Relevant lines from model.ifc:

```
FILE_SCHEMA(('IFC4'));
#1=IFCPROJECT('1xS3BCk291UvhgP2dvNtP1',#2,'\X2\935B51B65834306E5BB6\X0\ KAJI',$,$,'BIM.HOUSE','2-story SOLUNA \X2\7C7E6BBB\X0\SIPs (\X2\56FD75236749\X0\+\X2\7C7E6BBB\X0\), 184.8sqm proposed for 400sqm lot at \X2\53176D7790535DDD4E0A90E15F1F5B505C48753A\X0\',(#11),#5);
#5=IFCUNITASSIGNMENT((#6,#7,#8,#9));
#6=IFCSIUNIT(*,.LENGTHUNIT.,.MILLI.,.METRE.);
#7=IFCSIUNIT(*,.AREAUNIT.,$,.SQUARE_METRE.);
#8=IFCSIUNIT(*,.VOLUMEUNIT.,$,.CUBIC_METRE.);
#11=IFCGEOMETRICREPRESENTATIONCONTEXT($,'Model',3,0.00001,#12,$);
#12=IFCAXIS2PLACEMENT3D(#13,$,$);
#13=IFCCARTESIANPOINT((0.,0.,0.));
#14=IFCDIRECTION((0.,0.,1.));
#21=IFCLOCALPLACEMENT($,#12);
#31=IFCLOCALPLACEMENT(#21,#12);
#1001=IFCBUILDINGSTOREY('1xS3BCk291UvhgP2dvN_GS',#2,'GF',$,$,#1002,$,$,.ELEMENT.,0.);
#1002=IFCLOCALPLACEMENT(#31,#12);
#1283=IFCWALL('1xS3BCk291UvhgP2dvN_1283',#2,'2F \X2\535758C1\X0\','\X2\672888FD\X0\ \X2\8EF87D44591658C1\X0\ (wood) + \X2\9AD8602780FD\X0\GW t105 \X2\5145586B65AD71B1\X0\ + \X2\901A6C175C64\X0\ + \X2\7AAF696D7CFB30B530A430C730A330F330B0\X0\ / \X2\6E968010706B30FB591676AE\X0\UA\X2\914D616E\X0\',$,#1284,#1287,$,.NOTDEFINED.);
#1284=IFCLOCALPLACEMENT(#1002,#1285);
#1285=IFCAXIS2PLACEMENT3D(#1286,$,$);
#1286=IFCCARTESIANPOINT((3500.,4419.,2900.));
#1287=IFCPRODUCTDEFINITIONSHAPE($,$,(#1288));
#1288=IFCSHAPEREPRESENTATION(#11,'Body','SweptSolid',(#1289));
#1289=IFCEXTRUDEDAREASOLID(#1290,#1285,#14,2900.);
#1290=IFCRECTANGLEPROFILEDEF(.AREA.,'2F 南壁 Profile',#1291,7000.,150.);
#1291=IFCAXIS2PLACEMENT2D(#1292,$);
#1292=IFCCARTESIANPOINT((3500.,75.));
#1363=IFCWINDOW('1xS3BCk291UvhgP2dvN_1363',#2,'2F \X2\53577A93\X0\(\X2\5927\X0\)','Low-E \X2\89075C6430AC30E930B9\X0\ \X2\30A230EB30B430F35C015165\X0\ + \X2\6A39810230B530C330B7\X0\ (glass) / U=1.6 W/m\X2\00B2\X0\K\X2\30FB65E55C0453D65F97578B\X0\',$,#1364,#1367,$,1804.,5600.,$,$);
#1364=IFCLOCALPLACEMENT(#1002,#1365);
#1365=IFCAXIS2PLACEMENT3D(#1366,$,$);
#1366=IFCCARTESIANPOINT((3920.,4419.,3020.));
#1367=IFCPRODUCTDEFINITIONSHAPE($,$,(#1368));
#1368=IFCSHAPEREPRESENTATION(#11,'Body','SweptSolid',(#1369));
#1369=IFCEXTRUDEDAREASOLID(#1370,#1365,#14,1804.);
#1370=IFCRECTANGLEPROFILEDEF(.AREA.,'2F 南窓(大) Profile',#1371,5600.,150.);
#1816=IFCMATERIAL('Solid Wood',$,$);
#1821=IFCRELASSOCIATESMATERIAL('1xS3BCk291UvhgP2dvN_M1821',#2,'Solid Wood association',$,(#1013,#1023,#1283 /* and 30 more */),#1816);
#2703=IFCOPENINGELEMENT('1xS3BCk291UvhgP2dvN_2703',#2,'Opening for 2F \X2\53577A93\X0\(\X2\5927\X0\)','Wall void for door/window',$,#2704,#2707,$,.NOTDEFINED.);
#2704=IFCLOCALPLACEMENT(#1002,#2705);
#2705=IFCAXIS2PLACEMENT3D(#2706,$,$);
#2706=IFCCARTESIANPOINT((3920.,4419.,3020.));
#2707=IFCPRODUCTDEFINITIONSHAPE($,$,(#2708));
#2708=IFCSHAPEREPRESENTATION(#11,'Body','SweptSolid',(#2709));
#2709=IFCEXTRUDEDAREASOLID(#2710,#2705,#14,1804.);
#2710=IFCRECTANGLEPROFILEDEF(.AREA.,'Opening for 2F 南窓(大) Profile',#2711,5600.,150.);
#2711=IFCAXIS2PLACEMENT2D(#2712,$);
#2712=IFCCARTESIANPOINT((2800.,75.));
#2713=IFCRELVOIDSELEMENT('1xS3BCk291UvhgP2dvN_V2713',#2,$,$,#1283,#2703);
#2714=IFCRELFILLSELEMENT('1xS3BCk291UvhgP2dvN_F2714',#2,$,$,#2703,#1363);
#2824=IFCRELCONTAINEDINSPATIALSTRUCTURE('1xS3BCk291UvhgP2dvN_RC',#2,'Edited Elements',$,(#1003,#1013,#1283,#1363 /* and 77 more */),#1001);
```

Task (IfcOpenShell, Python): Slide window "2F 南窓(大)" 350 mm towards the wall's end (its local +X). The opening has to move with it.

```python
import ifcopenshell
import ifcopenshell.api.geometry
import ifcopenshell.util.placement
import ifcopenshell.util.unit

model = ifcopenshell.open("model.ifc")
unit_scale = ifcopenshell.util.unit.calculate_unit_scale(model)

window = model.by_guid("1xS3BCk291UvhgP2dvN_1363")
opening = window.FillsVoids[0].RelatingOpeningElement
wall = opening.VoidsElements[0].RelatingBuildingElement

wall_matrix = ifcopenshell.util.placement.get_local_placement(wall.ObjectPlacement)
shift = wall_matrix[:3, 0] * 0.35 / unit_scale
before = ifcopenshell.util.placement.get_local_placement(window.ObjectPlacement)[:3, 3].copy()

# The window is not placed relative to its opening, so move both.
for product in (opening, window):
    matrix = ifcopenshell.util.placement.get_local_placement(product.ObjectPlacement)
    matrix[:3, 3] += shift
    ifcopenshell.api.geometry.edit_object_placement(model, product=product, matrix=matrix, is_si=False)

after = ifcopenshell.util.placement.get_local_placement(window.ObjectPlacement)[:3, 3]
print("window moved by", (after - before).round(3) + 0.0)

model.write("model-out.ifc")
```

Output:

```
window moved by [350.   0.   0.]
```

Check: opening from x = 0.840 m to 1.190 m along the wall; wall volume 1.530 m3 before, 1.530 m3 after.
